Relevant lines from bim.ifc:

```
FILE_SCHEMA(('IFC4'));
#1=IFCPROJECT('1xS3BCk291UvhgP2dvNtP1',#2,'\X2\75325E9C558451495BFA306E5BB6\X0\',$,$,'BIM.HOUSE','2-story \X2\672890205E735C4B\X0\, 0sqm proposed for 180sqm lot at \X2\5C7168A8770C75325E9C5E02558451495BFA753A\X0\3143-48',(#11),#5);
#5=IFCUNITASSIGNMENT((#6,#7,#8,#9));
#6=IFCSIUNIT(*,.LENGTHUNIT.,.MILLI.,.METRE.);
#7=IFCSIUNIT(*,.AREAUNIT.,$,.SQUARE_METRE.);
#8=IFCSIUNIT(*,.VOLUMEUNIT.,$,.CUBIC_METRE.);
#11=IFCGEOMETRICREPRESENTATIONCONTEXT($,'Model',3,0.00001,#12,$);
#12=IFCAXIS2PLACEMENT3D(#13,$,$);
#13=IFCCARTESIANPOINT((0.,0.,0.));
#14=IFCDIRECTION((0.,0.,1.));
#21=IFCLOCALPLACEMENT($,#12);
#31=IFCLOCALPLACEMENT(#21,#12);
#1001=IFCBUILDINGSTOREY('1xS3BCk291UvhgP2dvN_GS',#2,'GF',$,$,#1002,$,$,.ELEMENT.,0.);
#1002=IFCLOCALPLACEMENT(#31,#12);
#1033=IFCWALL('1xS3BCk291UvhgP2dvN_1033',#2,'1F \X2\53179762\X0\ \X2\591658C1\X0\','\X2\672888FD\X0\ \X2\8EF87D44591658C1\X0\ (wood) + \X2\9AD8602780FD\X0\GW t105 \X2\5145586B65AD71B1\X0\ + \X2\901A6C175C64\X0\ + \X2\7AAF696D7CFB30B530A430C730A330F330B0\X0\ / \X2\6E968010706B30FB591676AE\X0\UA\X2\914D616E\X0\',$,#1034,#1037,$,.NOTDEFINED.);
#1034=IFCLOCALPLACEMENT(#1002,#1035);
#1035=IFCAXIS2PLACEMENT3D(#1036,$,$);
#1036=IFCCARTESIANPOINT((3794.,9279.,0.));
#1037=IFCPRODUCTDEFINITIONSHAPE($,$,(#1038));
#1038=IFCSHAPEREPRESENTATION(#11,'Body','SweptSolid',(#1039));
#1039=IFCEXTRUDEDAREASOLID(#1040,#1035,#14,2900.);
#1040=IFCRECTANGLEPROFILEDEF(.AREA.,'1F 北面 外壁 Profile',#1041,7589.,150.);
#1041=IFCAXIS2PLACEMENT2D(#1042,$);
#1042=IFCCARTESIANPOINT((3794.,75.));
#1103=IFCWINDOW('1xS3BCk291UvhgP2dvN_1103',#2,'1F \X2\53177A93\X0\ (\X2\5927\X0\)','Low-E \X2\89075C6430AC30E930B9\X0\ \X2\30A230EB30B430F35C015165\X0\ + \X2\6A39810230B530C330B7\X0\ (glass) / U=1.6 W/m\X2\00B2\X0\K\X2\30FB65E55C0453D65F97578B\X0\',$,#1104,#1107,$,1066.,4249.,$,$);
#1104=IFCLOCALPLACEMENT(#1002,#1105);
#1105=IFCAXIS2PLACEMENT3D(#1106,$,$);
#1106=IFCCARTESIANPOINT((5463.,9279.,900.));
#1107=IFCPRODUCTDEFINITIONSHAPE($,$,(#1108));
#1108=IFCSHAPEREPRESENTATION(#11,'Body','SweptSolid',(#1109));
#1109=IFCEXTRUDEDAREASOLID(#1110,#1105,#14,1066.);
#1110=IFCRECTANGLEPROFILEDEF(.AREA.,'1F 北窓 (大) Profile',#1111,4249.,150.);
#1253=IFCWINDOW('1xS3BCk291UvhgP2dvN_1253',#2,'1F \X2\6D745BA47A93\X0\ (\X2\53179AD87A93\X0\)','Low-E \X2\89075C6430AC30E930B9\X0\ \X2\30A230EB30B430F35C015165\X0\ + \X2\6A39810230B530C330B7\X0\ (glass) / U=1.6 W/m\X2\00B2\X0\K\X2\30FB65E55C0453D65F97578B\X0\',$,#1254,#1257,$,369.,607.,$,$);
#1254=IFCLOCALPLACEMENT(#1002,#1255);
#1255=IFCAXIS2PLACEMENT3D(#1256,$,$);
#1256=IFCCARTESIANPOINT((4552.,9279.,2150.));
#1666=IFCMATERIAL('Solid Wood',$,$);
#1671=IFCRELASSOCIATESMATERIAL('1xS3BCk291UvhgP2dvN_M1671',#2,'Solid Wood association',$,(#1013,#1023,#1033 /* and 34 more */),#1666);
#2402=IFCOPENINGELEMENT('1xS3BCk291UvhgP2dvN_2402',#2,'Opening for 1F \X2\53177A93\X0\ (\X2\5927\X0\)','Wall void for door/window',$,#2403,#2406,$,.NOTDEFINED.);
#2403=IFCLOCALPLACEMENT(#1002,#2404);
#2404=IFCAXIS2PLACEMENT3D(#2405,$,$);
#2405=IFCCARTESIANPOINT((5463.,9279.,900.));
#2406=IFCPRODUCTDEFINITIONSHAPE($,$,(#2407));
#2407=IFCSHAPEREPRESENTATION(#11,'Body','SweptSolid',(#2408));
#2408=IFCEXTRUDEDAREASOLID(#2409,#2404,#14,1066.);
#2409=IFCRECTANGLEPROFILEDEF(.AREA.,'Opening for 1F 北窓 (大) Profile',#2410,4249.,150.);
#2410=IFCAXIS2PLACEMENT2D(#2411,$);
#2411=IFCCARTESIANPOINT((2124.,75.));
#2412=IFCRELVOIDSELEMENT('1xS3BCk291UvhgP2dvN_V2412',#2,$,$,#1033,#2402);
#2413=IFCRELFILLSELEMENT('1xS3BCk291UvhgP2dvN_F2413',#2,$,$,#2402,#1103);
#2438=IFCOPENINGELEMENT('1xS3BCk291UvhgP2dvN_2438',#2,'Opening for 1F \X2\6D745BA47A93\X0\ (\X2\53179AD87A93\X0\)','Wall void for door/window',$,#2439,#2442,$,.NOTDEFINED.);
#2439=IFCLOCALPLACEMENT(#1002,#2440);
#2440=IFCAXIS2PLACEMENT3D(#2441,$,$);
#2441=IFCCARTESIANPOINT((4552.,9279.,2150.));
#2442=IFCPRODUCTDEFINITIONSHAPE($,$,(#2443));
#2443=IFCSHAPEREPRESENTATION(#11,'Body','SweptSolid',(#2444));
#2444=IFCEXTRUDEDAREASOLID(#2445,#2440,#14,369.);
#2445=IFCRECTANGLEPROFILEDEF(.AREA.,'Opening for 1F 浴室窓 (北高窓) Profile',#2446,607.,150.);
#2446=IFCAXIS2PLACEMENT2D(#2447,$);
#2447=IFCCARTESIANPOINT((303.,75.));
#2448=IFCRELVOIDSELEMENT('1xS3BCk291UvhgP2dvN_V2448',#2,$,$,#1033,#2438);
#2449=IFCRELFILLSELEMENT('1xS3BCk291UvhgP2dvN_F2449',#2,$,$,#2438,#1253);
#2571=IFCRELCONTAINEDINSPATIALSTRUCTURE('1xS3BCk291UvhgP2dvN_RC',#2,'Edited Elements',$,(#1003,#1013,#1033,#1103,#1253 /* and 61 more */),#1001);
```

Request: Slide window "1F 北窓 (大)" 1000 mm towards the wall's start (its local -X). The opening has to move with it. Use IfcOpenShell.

```python
import ifcopenshell
import ifcopenshell.api.geometry
import ifcopenshell.util.placement
import ifcopenshell.util.unit

model = ifcopenshell.open("bim.ifc")
unit_scale = ifcopenshell.util.unit.calculate_unit_scale(model)

window = model.by_id(1103)
opening = window.FillsVoids[0].RelatingOpeningElement
wall = opening.VoidsElements[0].RelatingBuildingElement

wall_matrix = ifcopenshell.util.placement.get_local_placement(wall.ObjectPlacement)
shift = wall_matrix[:3, 0] * -1 / unit_scale
before = ifcopenshell.util.placement.get_local_placement(window.ObjectPlacement)[:3, 3].copy()

# The window is not placed relative to its opening, so move both.
for product in (opening, window):
    matrix = ifcopenshell.util.placement.get_local_placement(product.ObjectPlacement)
    matrix[:3, 3] += shift
    ifcopenshell.api.geometry.edit_object_placement(model, product=product, matrix=matrix, is_si=False)

after = ifcopenshell.util.placement.get_local_placement(window.ObjectPlacement)[:3, 3]
print("window moved by", (after - before).round(3) + 0.0)

model.write("bim-out.ifc")
```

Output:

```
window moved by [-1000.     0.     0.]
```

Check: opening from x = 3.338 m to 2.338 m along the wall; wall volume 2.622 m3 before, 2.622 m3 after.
